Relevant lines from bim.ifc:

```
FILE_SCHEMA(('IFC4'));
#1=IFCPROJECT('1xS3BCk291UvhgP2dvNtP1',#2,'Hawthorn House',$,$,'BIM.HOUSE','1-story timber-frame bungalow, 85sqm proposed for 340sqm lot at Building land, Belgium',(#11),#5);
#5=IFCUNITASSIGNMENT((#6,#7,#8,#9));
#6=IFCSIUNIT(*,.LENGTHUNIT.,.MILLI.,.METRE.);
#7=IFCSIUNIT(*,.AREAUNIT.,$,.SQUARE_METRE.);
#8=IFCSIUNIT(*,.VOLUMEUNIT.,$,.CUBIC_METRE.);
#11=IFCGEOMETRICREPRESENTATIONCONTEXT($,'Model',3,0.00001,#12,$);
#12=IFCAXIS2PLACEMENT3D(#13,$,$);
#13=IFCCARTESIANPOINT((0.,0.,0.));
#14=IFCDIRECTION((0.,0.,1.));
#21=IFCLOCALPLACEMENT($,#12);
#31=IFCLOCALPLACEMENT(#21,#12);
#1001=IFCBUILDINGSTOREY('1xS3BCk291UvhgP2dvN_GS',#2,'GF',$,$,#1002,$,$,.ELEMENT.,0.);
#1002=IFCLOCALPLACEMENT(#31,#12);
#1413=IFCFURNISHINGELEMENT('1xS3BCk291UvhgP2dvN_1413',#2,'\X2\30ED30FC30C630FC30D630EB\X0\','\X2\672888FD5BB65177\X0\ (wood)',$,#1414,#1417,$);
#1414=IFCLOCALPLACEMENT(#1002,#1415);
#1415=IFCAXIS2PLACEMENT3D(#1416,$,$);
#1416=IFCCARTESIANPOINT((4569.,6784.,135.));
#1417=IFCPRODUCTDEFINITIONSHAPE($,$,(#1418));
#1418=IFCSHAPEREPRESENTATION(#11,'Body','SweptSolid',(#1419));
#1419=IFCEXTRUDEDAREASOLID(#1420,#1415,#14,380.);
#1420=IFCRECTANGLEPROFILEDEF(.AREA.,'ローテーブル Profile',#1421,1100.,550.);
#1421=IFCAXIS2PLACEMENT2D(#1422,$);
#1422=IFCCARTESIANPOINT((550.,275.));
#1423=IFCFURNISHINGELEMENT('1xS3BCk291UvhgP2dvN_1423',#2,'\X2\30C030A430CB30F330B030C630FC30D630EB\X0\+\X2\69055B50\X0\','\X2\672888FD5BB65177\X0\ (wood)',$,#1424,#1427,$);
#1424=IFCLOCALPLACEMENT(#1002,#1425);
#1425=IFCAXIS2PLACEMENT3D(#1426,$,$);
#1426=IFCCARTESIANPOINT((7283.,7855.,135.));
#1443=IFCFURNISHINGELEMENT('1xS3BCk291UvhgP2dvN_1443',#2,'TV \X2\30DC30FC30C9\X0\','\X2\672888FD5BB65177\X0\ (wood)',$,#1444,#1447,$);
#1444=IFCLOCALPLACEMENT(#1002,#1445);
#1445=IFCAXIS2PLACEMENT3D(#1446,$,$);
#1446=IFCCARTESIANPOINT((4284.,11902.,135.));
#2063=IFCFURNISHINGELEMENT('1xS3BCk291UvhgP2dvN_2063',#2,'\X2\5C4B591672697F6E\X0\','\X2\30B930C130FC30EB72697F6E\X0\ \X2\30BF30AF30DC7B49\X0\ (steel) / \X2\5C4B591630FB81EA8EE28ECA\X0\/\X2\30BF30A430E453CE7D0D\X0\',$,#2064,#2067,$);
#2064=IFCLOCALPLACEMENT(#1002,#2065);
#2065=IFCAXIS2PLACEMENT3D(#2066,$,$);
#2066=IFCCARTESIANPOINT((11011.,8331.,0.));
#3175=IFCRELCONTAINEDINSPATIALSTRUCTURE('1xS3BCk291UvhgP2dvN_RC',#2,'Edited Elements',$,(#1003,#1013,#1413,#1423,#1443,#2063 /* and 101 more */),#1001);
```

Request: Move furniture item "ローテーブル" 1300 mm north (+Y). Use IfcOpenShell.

```python
import ifcopenshell
import ifcopenshell.api.geometry
import ifcopenshell.util.placement
import ifcopenshell.util.unit

model = ifcopenshell.open("bim.ifc")
unit_scale = ifcopenshell.util.unit.calculate_unit_scale(model)

item = model.by_guid("1xS3BCk291UvhgP2dvN_1413")
matrix = ifcopenshell.util.placement.get_local_placement(item.ObjectPlacement)
matrix[1, 3] += 1.3 / unit_scale
ifcopenshell.api.geometry.edit_object_placement(model, product=item, matrix=matrix, is_si=False)

print(ifcopenshell.util.placement.get_local_placement(item.ObjectPlacement).round(3) + 0.0)

model.write("bim_v2.ifc")
```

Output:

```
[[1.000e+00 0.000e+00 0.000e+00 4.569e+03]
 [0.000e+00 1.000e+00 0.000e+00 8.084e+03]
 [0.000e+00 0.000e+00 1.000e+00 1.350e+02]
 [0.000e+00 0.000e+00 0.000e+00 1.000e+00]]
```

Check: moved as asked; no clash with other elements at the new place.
